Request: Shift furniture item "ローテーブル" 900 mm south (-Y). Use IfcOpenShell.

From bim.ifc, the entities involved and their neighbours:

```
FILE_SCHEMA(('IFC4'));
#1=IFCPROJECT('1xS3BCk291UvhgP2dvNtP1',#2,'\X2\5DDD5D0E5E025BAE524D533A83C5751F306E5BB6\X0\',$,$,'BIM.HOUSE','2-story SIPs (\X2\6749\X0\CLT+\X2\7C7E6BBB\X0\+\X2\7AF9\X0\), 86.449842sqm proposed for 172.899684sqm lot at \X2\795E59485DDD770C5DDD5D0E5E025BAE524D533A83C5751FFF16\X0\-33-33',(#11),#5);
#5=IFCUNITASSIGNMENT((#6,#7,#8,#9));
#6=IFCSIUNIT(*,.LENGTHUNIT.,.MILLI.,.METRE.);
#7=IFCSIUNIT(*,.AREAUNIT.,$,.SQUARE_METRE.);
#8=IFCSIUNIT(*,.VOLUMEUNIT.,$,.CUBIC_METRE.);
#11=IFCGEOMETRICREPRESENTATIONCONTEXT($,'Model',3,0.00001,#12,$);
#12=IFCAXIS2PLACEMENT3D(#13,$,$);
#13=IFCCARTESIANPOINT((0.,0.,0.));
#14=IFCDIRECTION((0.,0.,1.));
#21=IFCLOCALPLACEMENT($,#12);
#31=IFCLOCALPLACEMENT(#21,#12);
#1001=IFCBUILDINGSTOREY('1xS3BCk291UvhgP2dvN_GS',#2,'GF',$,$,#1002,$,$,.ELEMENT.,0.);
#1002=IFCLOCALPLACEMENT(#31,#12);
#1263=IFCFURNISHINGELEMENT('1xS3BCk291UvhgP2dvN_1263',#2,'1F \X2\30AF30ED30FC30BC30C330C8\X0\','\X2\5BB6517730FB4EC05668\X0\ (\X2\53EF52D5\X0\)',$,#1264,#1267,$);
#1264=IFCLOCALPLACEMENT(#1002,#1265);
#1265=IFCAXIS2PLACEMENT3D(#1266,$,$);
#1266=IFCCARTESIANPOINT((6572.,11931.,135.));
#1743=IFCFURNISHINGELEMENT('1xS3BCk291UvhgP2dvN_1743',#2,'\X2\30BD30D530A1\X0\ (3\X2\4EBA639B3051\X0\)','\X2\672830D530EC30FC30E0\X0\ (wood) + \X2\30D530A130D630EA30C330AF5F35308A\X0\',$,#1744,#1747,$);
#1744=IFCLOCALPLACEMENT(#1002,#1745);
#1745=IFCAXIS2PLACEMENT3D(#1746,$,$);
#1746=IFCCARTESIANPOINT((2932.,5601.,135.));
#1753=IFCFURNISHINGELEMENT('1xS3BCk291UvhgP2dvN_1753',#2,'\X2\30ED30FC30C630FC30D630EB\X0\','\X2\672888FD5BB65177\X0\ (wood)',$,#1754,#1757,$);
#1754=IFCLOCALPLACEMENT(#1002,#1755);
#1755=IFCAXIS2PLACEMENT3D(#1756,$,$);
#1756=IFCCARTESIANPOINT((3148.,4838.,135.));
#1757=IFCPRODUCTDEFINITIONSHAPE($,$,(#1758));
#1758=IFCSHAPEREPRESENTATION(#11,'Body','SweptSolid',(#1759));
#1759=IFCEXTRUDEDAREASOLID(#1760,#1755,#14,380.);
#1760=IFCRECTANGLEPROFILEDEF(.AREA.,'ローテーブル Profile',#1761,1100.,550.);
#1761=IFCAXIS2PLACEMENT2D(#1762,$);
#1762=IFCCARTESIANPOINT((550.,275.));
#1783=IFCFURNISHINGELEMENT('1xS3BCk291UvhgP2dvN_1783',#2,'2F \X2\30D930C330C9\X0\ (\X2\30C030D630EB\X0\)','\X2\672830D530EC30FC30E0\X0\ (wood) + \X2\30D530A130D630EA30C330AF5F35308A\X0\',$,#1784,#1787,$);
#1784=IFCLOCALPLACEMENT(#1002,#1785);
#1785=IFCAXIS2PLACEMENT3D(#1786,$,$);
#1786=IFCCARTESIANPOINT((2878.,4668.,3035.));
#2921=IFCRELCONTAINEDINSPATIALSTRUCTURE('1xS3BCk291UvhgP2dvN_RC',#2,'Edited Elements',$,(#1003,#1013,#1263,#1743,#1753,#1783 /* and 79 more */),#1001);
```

```python
import ifcopenshell
import ifcopenshell.api.geometry
import ifcopenshell.util.placement
import ifcopenshell.util.unit

model = ifcopenshell.open("bim.ifc")
unit_scale = ifcopenshell.util.unit.calculate_unit_scale(model)

item = model.by_id(1753)
matrix = ifcopenshell.util.placement.get_local_placement(item.ObjectPlacement)
matrix[1, 3] -= 0.9 / unit_scale
ifcopenshell.api.geometry.edit_object_placement(model, product=item, matrix=matrix, is_si=False)

print(ifcopenshell.util.placement.get_local_placement(item.ObjectPlacement).round(3) + 0.0)

model.write("bim-out.ifc")
```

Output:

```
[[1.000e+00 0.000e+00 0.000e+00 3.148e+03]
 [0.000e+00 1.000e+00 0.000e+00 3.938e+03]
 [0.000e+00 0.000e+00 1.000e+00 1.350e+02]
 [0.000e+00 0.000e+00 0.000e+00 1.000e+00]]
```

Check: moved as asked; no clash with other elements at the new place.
